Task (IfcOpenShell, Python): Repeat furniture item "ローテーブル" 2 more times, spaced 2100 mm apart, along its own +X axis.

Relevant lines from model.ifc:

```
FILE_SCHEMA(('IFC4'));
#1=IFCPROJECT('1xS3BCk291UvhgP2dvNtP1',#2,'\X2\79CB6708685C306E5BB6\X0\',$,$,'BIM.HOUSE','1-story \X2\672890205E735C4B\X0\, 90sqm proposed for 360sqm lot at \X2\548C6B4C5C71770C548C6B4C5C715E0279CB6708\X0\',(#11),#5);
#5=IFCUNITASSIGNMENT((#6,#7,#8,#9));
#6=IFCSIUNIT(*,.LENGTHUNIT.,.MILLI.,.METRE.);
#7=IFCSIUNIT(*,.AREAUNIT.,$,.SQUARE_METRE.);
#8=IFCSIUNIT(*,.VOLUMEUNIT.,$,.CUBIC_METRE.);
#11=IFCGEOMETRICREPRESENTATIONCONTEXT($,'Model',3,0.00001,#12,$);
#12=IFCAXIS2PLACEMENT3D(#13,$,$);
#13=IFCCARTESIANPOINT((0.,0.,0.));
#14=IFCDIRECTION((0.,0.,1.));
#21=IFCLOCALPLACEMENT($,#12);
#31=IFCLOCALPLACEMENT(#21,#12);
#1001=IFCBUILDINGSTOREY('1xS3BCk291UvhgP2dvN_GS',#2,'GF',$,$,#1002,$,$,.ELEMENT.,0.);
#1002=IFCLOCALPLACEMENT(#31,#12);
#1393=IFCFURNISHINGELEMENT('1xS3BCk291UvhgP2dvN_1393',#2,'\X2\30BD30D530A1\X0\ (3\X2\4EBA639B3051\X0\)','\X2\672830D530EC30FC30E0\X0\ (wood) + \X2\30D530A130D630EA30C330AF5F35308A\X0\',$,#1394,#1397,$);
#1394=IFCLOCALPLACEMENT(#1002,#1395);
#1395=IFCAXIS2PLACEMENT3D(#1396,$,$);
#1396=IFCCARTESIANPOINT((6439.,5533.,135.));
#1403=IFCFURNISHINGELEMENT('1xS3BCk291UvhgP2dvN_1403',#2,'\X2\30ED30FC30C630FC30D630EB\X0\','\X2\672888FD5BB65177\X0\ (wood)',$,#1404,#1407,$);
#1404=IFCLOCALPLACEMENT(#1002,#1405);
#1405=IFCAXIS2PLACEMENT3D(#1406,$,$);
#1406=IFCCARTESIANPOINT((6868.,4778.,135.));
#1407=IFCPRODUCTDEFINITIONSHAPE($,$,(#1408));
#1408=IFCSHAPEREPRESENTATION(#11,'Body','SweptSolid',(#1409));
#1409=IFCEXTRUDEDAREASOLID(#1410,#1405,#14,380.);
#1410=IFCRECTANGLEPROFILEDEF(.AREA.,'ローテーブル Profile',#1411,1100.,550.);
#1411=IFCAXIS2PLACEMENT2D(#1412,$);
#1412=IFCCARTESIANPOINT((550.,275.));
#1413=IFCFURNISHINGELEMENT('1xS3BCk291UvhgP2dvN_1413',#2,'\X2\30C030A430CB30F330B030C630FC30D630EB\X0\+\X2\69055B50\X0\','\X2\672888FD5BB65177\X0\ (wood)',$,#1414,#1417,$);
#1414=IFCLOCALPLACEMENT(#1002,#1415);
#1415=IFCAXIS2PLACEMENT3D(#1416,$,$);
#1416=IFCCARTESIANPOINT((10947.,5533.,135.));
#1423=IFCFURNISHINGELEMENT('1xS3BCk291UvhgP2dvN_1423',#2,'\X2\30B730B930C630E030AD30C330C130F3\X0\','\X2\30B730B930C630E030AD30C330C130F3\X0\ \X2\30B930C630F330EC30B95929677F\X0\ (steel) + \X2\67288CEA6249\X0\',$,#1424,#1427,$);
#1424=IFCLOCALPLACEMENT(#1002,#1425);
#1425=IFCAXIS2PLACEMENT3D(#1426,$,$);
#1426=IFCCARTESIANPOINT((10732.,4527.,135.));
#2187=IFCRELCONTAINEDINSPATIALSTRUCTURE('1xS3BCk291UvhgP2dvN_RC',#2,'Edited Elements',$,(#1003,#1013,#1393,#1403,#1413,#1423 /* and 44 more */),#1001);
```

```python
import ifcopenshell
import ifcopenshell.api.geometry
import ifcopenshell.api.root
import ifcopenshell.util.element
import ifcopenshell.util.placement

model = ifcopenshell.open("model.ifc")


def reuse_history(source, copy):
    """copy_class also copies each property set's owner history, people and application; keep the originals."""
    for rel in copy.IsDefinedBy:
        if rel.is_a("IfcRelDefinesByProperties") and (history := rel.RelatingPropertyDefinition.OwnerHistory):
            rel.RelatingPropertyDefinition.OwnerHistory = source.OwnerHistory
            ifcopenshell.util.element.remove_deep2(model, history)


source = model.by_guid("1xS3BCk291UvhgP2dvN_1403")
base = ifcopenshell.util.placement.get_local_placement(source.ObjectPlacement)
step = base[:3, 0] * 2100.0

for i in range(1, 3):
    copy = ifcopenshell.api.root.copy_class(model, product=source)
    copy.Representation = ifcopenshell.util.element.copy_deep(
        model, source.Representation, exclude=["IfcGeometricRepresentationContext", "IfcRepresentationMap"]
    )
    reuse_history(source, copy)
    matrix = base.copy()
    matrix[:3, 3] += i * step
    print("added at", matrix[:3, 3].round(3) + 0.0)
    ifcopenshell.api.geometry.edit_object_placement(model, product=copy, matrix=matrix, is_si=False)

model.write("model_updated.ifc")
```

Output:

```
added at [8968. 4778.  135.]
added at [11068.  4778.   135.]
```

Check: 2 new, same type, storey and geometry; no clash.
